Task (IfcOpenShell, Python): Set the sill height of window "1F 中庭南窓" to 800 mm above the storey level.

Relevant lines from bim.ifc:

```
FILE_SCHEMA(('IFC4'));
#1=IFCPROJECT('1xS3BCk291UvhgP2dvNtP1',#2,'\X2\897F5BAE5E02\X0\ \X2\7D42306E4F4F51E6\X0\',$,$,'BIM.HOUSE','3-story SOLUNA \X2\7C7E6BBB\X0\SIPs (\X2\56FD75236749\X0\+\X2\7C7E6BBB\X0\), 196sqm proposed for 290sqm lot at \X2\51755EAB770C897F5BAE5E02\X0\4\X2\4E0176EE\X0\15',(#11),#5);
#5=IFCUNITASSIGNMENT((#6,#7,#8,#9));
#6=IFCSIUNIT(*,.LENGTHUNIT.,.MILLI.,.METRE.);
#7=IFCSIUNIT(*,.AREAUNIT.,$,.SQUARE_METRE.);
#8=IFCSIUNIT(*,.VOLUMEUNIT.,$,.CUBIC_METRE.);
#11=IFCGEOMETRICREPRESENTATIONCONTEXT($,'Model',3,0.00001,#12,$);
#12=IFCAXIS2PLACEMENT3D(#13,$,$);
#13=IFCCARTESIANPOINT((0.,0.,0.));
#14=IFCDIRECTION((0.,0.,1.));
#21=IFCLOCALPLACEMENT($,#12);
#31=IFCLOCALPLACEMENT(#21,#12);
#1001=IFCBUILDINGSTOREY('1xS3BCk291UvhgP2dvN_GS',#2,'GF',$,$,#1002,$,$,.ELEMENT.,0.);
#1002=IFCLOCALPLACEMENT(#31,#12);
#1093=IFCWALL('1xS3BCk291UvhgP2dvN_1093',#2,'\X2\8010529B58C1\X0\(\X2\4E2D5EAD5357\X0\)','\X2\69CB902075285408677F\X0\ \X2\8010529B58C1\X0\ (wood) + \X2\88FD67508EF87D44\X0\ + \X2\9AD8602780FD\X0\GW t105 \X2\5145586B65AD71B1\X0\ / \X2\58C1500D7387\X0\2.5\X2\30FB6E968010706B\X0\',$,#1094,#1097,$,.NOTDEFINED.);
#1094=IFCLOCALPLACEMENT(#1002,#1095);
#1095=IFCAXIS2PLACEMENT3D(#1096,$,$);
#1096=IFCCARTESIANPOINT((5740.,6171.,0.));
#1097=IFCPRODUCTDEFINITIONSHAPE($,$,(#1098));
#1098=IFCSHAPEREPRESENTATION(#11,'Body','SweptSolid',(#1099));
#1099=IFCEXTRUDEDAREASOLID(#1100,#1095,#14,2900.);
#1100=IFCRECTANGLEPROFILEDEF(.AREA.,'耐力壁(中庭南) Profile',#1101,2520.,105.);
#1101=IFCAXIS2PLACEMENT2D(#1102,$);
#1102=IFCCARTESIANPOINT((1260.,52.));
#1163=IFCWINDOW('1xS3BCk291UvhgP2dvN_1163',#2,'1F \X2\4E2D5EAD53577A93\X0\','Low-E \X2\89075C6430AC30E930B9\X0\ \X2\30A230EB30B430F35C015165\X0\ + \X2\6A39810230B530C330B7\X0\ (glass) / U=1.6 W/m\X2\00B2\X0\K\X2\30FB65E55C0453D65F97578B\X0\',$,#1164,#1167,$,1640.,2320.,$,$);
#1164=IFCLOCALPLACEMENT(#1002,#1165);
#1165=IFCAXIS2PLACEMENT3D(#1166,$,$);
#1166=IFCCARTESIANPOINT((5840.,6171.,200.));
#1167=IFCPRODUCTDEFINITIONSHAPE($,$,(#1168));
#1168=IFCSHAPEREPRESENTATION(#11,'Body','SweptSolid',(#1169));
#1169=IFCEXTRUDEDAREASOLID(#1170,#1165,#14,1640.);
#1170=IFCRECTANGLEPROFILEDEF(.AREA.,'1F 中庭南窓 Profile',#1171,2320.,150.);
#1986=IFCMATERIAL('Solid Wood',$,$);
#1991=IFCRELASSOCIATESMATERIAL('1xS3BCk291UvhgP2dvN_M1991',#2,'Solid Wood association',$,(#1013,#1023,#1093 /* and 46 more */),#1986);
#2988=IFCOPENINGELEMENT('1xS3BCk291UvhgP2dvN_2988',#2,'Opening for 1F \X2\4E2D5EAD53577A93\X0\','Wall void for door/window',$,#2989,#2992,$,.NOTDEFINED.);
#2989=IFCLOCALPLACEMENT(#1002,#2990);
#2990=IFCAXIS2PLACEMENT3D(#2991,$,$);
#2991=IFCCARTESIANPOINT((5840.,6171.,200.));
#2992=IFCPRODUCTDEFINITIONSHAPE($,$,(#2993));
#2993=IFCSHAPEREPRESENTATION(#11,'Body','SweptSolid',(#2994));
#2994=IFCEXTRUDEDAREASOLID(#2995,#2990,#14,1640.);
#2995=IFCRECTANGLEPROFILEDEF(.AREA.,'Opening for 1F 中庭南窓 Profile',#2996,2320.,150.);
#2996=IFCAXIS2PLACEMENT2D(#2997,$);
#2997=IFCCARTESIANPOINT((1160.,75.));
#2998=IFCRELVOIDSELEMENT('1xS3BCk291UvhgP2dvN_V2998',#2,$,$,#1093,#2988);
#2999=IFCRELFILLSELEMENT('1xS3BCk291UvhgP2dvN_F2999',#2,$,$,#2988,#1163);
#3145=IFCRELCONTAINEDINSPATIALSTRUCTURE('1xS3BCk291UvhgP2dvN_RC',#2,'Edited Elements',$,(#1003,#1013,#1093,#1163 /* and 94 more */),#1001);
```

```python
import numpy as np
import ifcopenshell
import ifcopenshell.api.geometry
import ifcopenshell.geom
import ifcopenshell.util.element
import ifcopenshell.util.placement
import ifcopenshell.util.shape
import ifcopenshell.util.unit

model = ifcopenshell.open("bim.ifc")
unit_scale = ifcopenshell.util.unit.calculate_unit_scale(model)

window = model.by_guid("1xS3BCk291UvhgP2dvN_1163")
opening = window.FillsVoids[0].RelatingOpeningElement
storey = ifcopenshell.util.element.get_container(window, ifc_class="IfcBuildingStorey")
level = ifcopenshell.util.placement.get_local_placement(storey.ObjectPlacement)[2, 3]

# The opening's origin need not be at the sill, so measure its lowest point.
shape = ifcopenshell.geom.create_shape(ifcopenshell.geom.settings(), opening)
bottom = ifcopenshell.util.shape.get_shape_bottom_elevation(shape, shape.geometry) / unit_scale
dz = level + 0.8 / unit_scale - bottom

shift = np.array([0.0, 0.0, dz])
# The window is not placed relative to its opening, so move both.
for product in (opening, window):
    matrix = ifcopenshell.util.placement.get_local_placement(product.ObjectPlacement)
    matrix[:3, 3] += shift
    ifcopenshell.api.geometry.edit_object_placement(model, product=product, matrix=matrix, is_si=False)

print(f"moved by {dz * unit_scale:+.3f} m")

model.write("bim_updated.ifc")
```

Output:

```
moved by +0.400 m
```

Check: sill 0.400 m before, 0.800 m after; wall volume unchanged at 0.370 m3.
